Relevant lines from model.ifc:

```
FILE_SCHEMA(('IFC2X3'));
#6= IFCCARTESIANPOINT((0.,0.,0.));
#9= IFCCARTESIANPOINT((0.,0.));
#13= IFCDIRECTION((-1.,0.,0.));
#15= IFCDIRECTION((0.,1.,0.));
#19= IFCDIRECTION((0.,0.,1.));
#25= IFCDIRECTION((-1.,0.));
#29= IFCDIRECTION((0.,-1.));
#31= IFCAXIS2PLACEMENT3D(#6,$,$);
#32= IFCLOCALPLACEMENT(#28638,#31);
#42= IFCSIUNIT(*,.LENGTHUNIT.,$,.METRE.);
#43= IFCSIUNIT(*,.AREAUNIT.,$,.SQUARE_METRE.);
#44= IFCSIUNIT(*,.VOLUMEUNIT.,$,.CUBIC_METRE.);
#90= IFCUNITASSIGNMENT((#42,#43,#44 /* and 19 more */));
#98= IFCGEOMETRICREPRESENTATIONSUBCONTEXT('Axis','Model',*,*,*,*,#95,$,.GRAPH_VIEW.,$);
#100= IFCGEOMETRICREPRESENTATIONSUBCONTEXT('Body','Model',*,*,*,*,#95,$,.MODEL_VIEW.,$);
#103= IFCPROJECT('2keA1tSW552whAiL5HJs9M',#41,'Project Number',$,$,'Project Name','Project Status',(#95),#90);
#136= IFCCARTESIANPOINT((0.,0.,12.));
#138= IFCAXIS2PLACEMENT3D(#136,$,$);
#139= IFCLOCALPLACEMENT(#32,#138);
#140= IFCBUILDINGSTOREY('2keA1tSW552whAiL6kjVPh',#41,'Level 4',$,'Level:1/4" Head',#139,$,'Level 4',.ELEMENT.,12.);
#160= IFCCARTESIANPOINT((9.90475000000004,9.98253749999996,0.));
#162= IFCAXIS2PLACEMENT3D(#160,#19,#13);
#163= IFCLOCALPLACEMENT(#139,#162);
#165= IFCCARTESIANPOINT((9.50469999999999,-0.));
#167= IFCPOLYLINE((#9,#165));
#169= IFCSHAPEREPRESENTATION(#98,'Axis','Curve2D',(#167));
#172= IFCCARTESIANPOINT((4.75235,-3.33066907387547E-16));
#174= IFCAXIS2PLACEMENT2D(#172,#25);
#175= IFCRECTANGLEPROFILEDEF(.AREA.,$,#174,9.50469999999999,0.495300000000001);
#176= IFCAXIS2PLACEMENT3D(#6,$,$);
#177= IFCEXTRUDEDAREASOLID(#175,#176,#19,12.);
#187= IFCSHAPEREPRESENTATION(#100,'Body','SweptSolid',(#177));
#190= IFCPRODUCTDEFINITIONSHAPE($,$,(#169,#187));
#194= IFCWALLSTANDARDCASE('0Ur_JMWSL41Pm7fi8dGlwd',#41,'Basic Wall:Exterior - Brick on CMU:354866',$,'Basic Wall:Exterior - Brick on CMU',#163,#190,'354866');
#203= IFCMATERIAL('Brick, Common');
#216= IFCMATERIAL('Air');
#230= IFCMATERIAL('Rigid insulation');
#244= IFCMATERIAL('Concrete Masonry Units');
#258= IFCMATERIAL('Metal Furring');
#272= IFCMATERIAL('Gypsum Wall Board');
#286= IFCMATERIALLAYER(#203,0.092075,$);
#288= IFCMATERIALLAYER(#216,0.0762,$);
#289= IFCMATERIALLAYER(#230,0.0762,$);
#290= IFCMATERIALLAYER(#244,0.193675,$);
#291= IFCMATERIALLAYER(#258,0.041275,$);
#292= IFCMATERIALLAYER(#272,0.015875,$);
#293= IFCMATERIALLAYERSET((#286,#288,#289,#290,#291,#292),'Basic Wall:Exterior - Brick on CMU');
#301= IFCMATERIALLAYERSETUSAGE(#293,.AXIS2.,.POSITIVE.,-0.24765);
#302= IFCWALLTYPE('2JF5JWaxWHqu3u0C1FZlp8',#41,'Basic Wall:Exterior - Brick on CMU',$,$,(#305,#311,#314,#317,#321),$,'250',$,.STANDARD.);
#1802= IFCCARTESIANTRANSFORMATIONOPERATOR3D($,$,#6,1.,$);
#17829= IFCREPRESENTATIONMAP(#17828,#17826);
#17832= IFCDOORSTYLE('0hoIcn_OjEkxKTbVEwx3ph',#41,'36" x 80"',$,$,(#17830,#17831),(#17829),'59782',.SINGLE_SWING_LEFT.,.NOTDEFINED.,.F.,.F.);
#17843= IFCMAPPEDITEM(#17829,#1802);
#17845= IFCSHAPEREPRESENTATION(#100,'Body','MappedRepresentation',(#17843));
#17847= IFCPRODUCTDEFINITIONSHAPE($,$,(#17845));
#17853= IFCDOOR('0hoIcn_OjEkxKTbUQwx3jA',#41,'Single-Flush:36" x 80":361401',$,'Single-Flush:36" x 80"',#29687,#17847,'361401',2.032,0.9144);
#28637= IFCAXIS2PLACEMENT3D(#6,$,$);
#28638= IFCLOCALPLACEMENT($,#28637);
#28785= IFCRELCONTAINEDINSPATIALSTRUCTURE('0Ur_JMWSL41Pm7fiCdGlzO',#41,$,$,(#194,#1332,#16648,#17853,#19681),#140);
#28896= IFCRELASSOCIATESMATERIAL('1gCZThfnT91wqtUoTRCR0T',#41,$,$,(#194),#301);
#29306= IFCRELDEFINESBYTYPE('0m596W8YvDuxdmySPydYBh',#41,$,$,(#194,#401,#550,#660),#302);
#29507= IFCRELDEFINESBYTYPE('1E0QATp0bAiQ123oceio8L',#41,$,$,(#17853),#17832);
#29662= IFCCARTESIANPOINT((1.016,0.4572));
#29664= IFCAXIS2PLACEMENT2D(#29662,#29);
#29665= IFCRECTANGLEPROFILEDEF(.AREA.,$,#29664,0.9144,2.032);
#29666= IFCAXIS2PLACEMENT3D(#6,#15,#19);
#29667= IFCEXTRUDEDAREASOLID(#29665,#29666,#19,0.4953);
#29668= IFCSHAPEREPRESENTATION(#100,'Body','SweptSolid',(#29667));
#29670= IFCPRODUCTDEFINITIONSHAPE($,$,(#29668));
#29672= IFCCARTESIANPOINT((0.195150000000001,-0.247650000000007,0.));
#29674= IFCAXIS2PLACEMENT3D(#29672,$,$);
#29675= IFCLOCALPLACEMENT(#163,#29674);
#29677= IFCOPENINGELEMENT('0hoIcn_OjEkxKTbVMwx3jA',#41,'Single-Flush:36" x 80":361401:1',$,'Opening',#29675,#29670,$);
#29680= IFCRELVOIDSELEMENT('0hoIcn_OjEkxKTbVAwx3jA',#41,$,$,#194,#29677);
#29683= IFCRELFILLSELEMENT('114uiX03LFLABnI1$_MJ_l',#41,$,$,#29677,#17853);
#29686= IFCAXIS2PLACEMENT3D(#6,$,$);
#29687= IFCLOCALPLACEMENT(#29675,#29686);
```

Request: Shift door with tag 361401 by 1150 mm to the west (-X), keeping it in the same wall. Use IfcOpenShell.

```python
import ifcopenshell
import ifcopenshell.api.geometry
import ifcopenshell.util.placement
import ifcopenshell.util.unit

model = ifcopenshell.open("model.ifc")
unit_scale = ifcopenshell.util.unit.calculate_unit_scale(model)

door = model.by_guid("0hoIcn_OjEkxKTbUQwx3jA")
opening = door.FillsVoids[0].RelatingOpeningElement
wall = opening.VoidsElements[0].RelatingBuildingElement

wall_matrix = ifcopenshell.util.placement.get_local_placement(wall.ObjectPlacement)
shift = wall_matrix[:3, 0] * 1.15 / unit_scale
before = ifcopenshell.util.placement.get_local_placement(door.ObjectPlacement)[:3, 3].copy()

# The door is placed relative to its opening, so it follows when the opening moves.
matrix = ifcopenshell.util.placement.get_local_placement(opening.ObjectPlacement)
matrix[:3, 3] += shift
ifcopenshell.api.geometry.edit_object_placement(
    model, product=opening, matrix=matrix, is_si=False, should_transform_children=True
)

after = ifcopenshell.util.placement.get_local_placement(door.ObjectPlacement)[:3, 3]
print("door moved by", (after - before).round(3) + 0.0)

model.write("model_edited.ifc")
```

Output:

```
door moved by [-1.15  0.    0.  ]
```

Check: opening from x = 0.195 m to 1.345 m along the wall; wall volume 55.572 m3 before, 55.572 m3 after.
